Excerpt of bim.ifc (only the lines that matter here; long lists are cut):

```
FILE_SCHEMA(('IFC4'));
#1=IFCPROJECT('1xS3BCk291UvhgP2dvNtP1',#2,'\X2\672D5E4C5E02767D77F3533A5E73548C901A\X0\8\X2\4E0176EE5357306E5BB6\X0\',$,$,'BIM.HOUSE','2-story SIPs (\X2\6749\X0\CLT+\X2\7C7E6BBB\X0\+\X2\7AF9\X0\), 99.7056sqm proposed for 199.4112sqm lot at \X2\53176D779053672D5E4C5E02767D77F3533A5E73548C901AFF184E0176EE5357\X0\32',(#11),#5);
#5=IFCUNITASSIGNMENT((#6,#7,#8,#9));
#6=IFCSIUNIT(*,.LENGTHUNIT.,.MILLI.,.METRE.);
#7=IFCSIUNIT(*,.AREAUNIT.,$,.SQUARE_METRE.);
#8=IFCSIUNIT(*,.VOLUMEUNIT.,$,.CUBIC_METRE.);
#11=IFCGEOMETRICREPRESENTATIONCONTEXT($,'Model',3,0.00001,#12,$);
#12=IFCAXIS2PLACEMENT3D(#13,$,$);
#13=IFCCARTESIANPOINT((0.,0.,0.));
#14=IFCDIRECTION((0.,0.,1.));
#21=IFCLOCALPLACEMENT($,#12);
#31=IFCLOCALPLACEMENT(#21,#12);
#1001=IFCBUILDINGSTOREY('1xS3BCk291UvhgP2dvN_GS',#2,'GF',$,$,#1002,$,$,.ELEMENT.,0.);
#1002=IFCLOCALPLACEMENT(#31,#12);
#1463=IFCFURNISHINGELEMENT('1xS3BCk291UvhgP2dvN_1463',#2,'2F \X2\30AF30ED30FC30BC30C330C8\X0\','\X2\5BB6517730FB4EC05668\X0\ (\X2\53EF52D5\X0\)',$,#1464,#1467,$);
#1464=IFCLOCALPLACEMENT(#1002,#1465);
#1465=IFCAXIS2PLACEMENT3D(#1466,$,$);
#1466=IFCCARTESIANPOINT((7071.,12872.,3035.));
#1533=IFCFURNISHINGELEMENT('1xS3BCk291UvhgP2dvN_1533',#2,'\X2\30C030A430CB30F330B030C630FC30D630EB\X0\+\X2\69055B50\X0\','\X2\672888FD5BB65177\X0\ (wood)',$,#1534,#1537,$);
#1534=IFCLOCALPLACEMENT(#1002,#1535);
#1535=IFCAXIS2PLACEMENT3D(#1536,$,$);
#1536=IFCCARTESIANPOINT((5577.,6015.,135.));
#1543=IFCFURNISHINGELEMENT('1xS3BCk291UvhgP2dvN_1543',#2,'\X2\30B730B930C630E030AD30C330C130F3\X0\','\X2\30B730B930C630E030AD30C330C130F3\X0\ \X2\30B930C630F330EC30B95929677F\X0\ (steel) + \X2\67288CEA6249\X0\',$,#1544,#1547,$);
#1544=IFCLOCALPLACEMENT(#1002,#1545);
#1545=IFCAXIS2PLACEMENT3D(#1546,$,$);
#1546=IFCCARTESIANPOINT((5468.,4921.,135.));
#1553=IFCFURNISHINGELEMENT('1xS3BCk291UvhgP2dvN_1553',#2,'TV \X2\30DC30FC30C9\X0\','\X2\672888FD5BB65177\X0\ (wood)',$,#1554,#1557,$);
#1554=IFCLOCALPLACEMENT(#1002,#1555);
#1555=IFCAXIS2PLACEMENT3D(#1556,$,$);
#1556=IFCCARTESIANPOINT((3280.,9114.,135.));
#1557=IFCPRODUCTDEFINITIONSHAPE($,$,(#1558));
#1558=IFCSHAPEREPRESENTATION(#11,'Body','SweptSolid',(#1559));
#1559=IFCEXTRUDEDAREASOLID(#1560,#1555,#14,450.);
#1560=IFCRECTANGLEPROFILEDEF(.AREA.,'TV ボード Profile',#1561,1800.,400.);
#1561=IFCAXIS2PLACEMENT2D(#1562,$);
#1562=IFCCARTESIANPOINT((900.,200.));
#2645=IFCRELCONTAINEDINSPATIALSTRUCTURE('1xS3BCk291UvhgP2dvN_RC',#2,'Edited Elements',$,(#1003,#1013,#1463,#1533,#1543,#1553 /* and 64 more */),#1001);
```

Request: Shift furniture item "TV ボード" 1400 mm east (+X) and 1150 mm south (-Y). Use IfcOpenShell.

```python
import ifcopenshell
import ifcopenshell.api.geometry
import ifcopenshell.util.placement

model = ifcopenshell.open("bim.ifc")

item = model.by_guid("1xS3BCk291UvhgP2dvN_1553")
matrix = ifcopenshell.util.placement.get_local_placement(item.ObjectPlacement)
matrix[0, 3] += 1400.0
matrix[1, 3] -= 1150.0
ifcopenshell.api.geometry.edit_object_placement(model, product=item, matrix=matrix, is_si=False)

print(ifcopenshell.util.placement.get_local_placement(item.ObjectPlacement).round(3) + 0.0)

model.write("bim_edited.ifc")
```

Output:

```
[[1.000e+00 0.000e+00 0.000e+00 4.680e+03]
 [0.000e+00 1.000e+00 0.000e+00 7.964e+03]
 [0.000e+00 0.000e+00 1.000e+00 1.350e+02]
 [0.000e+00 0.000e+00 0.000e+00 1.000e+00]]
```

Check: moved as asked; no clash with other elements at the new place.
